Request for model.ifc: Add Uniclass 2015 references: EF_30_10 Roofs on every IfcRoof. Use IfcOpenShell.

First a look at what the model holds.

```python
import ifcopenshell

model = ifcopenshell.open("model.ifc")
print(model.schema)
print("classifications:", [c.Name for c in model.by_type("IfcClassification")])
for ifc_class in ("IfcDoor", "IfcRoof", "IfcStair", "IfcWall", "IfcWindow"):
    print(ifc_class, len(model.by_type(ifc_class)))
```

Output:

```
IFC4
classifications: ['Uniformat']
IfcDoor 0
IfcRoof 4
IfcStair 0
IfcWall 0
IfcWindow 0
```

```python
import ifcopenshell
import ifcopenshell.api.classification

model = ifcopenshell.open("model.ifc")

system = ifcopenshell.api.classification.add_classification(model, classification="Uniclass 2015")

codes = {
    "IfcRoof": ("EF_30_10", "Roofs"),
}
for ifc_class, (code, name) in codes.items():
    products = model.by_type(ifc_class)
    ifcopenshell.api.classification.add_reference(
        model, products=products, classification=system, identification=code, name=name
    )
    print(code, len(products))

model.write("model_v2.ifc")
```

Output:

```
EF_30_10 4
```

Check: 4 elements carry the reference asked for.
